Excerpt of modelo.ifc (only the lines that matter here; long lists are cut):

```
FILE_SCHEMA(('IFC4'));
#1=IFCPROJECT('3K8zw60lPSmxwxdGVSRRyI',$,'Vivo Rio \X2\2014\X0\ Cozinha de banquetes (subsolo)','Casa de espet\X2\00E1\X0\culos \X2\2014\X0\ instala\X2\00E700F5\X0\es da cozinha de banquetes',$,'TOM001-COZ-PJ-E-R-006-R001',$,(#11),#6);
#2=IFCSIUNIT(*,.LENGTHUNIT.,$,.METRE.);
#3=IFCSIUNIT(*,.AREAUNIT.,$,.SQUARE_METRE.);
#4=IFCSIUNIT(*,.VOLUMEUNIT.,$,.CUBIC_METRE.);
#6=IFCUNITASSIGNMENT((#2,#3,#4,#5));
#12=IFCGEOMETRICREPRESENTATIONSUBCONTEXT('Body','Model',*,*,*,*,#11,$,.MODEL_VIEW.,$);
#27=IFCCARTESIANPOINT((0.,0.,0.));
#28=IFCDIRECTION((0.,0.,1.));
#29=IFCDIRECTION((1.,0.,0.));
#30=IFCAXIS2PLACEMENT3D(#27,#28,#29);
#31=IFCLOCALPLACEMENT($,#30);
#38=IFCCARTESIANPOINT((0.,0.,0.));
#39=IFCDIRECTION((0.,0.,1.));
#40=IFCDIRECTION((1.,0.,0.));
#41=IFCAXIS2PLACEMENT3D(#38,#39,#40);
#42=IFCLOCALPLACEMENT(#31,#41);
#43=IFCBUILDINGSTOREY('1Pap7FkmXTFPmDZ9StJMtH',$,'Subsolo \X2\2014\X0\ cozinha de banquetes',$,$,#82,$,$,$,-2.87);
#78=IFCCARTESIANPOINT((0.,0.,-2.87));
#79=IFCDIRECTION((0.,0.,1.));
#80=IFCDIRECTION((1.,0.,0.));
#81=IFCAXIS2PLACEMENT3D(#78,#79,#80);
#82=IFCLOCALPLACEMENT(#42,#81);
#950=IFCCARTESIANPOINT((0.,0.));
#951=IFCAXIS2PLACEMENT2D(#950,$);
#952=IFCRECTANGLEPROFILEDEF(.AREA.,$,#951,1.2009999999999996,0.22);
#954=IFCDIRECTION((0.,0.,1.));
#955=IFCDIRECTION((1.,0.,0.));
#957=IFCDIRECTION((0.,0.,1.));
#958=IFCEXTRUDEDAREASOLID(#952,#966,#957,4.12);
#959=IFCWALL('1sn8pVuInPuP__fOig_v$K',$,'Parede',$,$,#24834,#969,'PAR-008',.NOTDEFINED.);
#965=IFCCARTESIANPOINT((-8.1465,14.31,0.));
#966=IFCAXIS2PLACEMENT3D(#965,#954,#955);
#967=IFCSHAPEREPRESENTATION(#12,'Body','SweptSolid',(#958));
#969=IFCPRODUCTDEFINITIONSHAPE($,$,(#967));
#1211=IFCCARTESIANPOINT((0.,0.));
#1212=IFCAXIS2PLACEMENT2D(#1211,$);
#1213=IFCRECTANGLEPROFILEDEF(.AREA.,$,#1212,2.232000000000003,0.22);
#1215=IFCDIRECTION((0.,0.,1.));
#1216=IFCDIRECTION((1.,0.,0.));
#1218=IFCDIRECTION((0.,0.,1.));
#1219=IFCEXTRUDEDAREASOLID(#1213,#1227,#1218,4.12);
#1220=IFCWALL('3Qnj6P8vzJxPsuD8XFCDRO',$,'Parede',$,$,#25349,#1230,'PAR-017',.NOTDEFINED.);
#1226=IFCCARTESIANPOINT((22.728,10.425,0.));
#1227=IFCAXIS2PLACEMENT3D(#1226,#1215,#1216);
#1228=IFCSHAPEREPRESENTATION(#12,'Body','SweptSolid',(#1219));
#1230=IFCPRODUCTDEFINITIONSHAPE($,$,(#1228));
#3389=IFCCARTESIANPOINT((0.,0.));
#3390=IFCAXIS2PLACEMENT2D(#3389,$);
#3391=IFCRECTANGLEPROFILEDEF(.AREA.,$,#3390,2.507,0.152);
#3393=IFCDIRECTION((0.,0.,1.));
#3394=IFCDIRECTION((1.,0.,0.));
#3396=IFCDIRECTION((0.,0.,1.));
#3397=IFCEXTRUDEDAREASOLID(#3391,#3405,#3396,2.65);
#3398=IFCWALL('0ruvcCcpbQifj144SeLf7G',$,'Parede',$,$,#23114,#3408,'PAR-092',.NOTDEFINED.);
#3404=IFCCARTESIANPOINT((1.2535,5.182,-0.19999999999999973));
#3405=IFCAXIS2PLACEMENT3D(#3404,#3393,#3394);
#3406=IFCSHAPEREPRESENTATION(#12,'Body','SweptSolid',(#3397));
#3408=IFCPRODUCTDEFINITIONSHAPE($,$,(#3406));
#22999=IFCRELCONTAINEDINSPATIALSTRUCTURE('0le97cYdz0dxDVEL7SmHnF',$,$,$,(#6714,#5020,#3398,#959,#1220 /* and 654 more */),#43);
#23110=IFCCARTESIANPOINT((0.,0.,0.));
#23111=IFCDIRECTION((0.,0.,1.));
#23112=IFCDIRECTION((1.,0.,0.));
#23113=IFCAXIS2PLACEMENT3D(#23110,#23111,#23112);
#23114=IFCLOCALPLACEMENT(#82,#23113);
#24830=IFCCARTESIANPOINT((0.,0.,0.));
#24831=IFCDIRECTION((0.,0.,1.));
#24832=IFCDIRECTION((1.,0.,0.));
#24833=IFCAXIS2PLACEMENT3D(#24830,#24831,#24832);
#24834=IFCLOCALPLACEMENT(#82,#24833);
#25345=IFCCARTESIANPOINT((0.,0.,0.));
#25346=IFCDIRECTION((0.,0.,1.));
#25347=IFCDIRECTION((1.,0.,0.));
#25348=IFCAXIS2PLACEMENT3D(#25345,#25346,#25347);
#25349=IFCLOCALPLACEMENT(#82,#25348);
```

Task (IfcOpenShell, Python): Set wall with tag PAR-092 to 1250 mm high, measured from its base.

```python
import ifcopenshell
import ifcopenshell.geom
import ifcopenshell.util.representation
import ifcopenshell.util.shape
import ifcopenshell.util.unit

model = ifcopenshell.open("modelo.ifc")
unit_scale = ifcopenshell.util.unit.calculate_unit_scale(model)
settings = ifcopenshell.geom.settings()


def volume(element):
    """Net volume in cubic metres, openings subtracted."""
    shape = ifcopenshell.geom.create_shape(settings, element)
    return ifcopenshell.util.shape.get_volume(shape.geometry)


wall = model.by_guid("0ruvcCcpbQifj144SeLf7G")
before = volume(wall)

body = ifcopenshell.util.representation.get_representation(wall, "Model", "Body")
solid = body.Items[0]
old_height = solid.Depth
solid.Depth = 1.25 / unit_scale
after = volume(wall)

print(f"height {old_height:g} -> {solid.Depth:g}, volume {before:.3f} -> {after:.3f} m3")

model.write("modelo_v2.ifc")
```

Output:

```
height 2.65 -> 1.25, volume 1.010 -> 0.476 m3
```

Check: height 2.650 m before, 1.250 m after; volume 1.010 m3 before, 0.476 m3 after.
